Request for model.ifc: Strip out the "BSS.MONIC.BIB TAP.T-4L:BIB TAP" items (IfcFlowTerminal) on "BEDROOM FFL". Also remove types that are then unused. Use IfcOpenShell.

First a look at what the model holds.

```python
import ifcopenshell
import ifcopenshell.util.element

model = ifcopenshell.open("model.ifc")
print(model.schema)
storey = next(s for s in model.by_type("IfcBuildingStorey") if s.Name == "BEDROOM FFL")
terminals = [e for e in ifcopenshell.util.element.get_decomposition(storey) if e.is_a("IfcFlowTerminal")]
seen = {}
for e in terminals:
    element_type = ifcopenshell.util.element.get_type(e)
    name = element_type.Name if element_type not in (None, e) else None
    seen[name] = seen.get(name, 0) + 1
for name, count in sorted(seen.items(), key=str):
    print(count, "x", name)
```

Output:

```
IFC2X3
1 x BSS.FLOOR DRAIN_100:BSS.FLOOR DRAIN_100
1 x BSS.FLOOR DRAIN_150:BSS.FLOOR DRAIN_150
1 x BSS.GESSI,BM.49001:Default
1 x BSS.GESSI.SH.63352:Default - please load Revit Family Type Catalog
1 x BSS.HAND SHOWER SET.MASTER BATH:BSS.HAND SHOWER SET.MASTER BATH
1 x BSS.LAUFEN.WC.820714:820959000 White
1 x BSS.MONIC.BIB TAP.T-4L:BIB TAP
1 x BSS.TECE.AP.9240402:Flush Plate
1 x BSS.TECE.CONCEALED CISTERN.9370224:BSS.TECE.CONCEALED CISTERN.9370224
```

```python
import ifcopenshell
import ifcopenshell.api.root
import ifcopenshell.util.element

model = ifcopenshell.open("model.ifc")

storey = next(s for s in model.by_type("IfcBuildingStorey") if s.Name == "BEDROOM FFL")
terminals = [e for e in ifcopenshell.util.element.get_decomposition(storey) if e.is_a("IfcFlowTerminal")]
targets = [e for e in terminals if (t := ifcopenshell.util.element.get_type(e)) not in (None, e) and t.Name == "BSS.MONIC.BIB TAP.T-4L:BIB TAP"]
types = {ifcopenshell.util.element.get_type(e) for e in targets} - {None, *targets}

for e in targets:
    ifcopenshell.api.root.remove_product(model, product=e)
print(len(targets), "removed")

unused = [t for t in types if not ifcopenshell.util.element.get_types(t)]
for t in unused:
    ifcopenshell.api.root.remove_product(model, product=t)
print(len(unused), "unused types removed")

model.write("model_rev.ifc")
```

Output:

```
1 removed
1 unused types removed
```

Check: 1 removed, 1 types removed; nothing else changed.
